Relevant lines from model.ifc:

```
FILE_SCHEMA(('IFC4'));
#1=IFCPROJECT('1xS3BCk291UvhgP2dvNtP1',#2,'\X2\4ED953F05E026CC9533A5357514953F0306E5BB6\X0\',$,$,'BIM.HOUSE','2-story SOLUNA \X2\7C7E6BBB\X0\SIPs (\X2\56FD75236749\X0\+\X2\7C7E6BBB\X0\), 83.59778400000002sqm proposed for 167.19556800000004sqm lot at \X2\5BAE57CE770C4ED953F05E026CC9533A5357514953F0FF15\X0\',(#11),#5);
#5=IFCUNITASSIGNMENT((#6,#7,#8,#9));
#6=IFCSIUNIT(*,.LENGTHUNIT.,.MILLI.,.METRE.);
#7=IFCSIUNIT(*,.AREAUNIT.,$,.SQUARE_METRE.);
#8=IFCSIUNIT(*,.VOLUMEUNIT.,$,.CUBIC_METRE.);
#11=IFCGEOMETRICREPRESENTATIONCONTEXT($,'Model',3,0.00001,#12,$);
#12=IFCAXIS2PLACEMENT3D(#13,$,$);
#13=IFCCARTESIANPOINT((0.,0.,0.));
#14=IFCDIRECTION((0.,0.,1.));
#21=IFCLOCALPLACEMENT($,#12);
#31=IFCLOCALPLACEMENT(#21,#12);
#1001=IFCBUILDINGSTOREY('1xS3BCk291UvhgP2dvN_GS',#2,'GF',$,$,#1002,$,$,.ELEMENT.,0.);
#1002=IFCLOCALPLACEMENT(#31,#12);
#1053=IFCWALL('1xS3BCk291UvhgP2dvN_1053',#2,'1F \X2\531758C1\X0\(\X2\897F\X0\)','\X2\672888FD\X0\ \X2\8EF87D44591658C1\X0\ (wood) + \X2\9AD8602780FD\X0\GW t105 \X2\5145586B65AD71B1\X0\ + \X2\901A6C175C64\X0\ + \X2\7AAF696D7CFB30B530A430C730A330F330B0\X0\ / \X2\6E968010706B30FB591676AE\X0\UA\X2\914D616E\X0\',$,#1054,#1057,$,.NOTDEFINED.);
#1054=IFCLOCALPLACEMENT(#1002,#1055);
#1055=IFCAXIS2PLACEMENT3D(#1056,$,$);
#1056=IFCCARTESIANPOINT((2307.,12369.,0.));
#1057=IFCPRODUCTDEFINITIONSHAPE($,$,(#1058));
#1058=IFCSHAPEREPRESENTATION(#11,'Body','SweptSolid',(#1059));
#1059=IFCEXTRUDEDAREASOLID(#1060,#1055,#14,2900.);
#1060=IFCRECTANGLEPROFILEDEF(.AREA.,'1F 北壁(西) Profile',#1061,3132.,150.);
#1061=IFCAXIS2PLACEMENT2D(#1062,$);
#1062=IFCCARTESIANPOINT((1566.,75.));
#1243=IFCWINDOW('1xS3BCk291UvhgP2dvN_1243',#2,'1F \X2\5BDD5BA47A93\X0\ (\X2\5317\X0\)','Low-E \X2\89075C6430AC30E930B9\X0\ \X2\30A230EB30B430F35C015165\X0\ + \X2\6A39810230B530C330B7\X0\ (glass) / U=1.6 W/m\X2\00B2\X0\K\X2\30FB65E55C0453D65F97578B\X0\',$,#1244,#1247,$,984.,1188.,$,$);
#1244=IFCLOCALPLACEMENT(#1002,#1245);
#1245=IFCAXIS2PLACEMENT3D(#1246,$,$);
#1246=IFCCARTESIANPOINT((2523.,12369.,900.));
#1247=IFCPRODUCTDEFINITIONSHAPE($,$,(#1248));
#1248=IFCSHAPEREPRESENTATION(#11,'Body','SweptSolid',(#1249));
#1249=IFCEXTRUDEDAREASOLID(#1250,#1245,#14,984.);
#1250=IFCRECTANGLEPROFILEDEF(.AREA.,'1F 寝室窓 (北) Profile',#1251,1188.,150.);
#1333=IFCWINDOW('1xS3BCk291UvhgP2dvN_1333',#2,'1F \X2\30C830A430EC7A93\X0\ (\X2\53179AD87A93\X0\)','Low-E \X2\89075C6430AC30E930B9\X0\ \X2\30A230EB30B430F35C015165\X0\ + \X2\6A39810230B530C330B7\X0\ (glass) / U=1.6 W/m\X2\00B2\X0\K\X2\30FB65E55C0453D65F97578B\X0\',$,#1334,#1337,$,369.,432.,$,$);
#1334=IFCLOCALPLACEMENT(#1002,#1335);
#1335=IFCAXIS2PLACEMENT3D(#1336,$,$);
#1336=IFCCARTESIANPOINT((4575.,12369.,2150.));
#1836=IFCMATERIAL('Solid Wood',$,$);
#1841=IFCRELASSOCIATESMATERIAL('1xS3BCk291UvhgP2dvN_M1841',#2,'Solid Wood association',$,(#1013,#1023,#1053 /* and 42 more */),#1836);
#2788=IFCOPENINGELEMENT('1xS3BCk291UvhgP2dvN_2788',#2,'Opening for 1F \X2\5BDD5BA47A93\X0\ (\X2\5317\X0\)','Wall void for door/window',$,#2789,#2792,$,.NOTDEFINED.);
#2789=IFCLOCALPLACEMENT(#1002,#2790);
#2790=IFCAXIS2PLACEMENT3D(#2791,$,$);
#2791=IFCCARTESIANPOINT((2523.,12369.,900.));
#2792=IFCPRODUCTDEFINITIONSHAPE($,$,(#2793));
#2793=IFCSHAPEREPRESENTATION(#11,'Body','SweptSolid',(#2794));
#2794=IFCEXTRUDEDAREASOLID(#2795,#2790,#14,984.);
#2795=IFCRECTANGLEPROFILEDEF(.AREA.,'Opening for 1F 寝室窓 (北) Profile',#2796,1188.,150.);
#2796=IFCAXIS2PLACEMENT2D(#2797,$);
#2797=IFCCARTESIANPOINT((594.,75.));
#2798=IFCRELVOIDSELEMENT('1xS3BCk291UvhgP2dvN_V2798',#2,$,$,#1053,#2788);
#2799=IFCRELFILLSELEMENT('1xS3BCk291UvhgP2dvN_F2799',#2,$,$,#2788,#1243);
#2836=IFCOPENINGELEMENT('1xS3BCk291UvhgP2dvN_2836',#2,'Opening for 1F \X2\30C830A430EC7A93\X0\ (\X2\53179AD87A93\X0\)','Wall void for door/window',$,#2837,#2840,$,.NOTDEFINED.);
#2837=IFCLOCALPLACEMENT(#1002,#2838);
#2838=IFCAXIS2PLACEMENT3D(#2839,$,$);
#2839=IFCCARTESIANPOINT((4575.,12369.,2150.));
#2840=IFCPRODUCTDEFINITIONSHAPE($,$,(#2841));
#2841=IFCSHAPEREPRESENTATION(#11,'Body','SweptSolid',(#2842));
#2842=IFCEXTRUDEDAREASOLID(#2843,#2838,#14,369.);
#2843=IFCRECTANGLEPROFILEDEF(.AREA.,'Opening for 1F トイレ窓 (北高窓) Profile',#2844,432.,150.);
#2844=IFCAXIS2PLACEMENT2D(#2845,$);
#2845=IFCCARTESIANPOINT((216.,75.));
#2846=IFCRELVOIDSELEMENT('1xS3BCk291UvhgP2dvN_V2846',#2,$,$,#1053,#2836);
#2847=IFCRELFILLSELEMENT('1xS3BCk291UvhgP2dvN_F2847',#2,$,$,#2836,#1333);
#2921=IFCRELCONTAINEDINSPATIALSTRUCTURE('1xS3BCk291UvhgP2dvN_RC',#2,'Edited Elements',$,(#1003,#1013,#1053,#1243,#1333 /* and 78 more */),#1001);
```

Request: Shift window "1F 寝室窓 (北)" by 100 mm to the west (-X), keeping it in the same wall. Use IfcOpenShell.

```python
import ifcopenshell
import ifcopenshell.api.geometry
import ifcopenshell.util.placement
import ifcopenshell.util.unit

model = ifcopenshell.open("model.ifc")
unit_scale = ifcopenshell.util.unit.calculate_unit_scale(model)

window = model.by_guid("1xS3BCk291UvhgP2dvN_1243")
opening = window.FillsVoids[0].RelatingOpeningElement
wall = opening.VoidsElements[0].RelatingBuildingElement

wall_matrix = ifcopenshell.util.placement.get_local_placement(wall.ObjectPlacement)
shift = wall_matrix[:3, 0] * -0.1 / unit_scale
before = ifcopenshell.util.placement.get_local_placement(window.ObjectPlacement)[:3, 3].copy()

# The window is not placed relative to its opening, so move both.
for product in (opening, window):
    matrix = ifcopenshell.util.placement.get_local_placement(product.ObjectPlacement)
    matrix[:3, 3] += shift
    ifcopenshell.api.geometry.edit_object_placement(model, product=product, matrix=matrix, is_si=False)

after = ifcopenshell.util.placement.get_local_placement(window.ObjectPlacement)[:3, 3]
print("window moved by", (after - before).round(3) + 0.0)

model.write("model_updated.ifc")
```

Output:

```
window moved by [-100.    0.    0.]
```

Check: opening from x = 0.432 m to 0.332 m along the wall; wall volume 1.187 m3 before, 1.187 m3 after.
